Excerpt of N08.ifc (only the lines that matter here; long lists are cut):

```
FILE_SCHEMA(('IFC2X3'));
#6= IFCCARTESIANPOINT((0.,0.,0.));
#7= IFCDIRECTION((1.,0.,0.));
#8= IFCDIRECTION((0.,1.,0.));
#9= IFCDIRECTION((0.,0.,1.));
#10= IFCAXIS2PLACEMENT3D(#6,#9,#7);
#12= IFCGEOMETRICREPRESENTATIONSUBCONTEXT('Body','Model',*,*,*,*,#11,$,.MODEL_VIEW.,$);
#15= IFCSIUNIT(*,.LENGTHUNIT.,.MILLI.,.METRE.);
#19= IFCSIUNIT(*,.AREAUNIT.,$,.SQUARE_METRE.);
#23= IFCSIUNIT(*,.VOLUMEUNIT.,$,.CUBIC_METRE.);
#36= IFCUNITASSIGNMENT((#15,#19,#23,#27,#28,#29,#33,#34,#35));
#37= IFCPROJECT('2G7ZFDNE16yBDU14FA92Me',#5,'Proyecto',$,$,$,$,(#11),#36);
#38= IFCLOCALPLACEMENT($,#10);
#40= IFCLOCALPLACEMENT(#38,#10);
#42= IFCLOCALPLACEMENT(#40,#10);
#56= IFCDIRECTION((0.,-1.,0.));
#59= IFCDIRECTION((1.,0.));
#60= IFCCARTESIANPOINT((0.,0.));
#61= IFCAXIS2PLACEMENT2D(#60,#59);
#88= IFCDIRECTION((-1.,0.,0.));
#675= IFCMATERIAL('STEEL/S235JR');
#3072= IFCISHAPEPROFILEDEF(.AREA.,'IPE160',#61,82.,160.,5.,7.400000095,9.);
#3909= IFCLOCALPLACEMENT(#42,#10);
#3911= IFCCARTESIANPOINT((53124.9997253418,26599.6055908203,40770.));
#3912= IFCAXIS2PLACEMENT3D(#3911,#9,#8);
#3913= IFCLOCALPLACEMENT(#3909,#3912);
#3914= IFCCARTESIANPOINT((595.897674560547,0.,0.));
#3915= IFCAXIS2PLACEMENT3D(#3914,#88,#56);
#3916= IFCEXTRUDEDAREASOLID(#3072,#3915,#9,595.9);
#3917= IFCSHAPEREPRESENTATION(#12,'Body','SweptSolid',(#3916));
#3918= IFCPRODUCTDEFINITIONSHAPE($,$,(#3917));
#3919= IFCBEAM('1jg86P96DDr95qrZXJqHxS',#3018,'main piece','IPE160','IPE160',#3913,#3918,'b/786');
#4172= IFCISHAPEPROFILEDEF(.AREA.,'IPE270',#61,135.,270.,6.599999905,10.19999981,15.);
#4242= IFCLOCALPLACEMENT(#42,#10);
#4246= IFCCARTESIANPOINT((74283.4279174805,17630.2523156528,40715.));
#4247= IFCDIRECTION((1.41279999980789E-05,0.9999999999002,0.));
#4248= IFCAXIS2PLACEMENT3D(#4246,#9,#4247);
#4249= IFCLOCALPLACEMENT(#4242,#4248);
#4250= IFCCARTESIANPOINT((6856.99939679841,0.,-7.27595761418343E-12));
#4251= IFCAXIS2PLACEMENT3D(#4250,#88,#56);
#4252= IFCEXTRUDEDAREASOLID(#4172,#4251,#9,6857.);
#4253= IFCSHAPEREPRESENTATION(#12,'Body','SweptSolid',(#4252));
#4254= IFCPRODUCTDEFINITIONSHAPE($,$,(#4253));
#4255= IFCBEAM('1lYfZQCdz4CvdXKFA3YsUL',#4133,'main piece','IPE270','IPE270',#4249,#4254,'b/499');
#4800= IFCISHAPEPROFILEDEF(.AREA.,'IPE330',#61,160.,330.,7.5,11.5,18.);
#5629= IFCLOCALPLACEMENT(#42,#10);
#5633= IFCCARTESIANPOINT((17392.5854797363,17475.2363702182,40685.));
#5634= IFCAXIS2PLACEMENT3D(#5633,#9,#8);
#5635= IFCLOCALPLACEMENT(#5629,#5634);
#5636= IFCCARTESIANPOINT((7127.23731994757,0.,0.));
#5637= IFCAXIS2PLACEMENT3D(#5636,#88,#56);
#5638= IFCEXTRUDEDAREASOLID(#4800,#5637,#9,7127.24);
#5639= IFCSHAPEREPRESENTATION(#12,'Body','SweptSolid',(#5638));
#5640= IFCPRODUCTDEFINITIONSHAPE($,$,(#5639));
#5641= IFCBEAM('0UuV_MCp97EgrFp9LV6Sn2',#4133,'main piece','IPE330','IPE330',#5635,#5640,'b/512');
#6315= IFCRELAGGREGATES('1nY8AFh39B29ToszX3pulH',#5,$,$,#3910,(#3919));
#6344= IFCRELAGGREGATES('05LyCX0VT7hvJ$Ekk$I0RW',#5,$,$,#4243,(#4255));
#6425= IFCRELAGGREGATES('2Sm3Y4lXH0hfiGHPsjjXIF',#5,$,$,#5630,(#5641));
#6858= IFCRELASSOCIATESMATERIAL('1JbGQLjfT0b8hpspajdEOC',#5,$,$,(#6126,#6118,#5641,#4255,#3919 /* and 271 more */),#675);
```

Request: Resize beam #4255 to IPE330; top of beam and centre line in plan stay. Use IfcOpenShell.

```python
import ifcopenshell
import ifcopenshell.util.element
import ifcopenshell.util.representation

model = ifcopenshell.open("N08.ifc")

member = model.by_id(4255)
source = next(p for p in model.by_type("IfcIShapeProfileDef") if p.ProfileName == "IPE330")

body = ifcopenshell.util.representation.get_representation(member, "Model", "Body")
solid = body.Items[0]
old_profile = solid.SweptArea

# Copy the section's sizes but keep this member's own profile position.
profile = ifcopenshell.util.element.copy(model, source)
# Profiles are centred, so shift by half the change in depth to hold the top.
shift = (old_profile.OverallDepth - profile.OverallDepth) / 2
x, y = old_profile.Position.Location.Coordinates
up = (0.0, 1.0)  # upwards, in the solid's own plane
location = model.createIfcCartesianPoint((x + up[0] * shift, y + up[1] * shift))
profile.Position = model.createIfcAxis2Placement2D(location, old_profile.Position.RefDirection)
solid.SweptArea = profile
if not model.get_total_inverses(old_profile):
    ifcopenshell.util.element.remove_deep2(model, old_profile)
member.Description = member.Description.replace("IPE270", "IPE330")
member.ObjectType = member.ObjectType.replace("IPE270", "IPE330")

print(solid.SweptArea)

model.write("N08_updated.ifc")
```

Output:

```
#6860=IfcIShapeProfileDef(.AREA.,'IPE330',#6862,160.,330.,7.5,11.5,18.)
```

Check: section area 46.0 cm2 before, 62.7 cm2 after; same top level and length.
